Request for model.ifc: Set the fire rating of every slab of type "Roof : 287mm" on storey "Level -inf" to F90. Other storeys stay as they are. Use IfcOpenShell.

First a look at what the model holds.

```python
import ifcopenshell
import ifcopenshell.util.element

model = ifcopenshell.open("model.ifc")
print(model.schema)
storey = next(s for s in model.by_type("IfcBuildingStorey") if s.Name == "Level -inf")
slabs = [e for e in ifcopenshell.util.element.get_decomposition(storey) if e.is_a("IfcSlab")]
seen = {}
for e in slabs:
    element_type = ifcopenshell.util.element.get_type(e)
    key = (element_type.Name if element_type != e and element_type else None, ifcopenshell.util.element.get_pset(e, "Pset_SlabCommon", "FireRating"))
    seen[key] = seen.get(key, 0) + 1
for (name, value), count in sorted(seen.items(), key=str):
    print(count, "x", name, "|", value)
```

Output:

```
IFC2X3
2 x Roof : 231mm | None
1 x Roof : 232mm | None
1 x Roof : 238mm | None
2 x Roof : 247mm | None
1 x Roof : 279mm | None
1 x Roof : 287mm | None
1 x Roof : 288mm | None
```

```python
import ifcopenshell
import ifcopenshell.api.pset
import ifcopenshell.util.element

model = ifcopenshell.open("model.ifc")

storey = next(s for s in model.by_type("IfcBuildingStorey") if s.Name == "Level -inf")
slabs = [e for e in ifcopenshell.util.element.get_decomposition(storey) if e.is_a("IfcSlab")]

count = 0
for e in slabs:
    element_type = ifcopenshell.util.element.get_type(e)
    if element_type in (None, e) or element_type.Name != "Roof : 287mm":
        continue
    # add_pset returns the element's existing set when there is one.
    pset = ifcopenshell.api.pset.add_pset(model, product=e, name="Pset_SlabCommon")
    ifcopenshell.api.pset.edit_pset(model, pset=pset, properties={"FireRating": "F90"})
    count += 1

print(count, "slabs updated")

model.write("model-out.ifc")
```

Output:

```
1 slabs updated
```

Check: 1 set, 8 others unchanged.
